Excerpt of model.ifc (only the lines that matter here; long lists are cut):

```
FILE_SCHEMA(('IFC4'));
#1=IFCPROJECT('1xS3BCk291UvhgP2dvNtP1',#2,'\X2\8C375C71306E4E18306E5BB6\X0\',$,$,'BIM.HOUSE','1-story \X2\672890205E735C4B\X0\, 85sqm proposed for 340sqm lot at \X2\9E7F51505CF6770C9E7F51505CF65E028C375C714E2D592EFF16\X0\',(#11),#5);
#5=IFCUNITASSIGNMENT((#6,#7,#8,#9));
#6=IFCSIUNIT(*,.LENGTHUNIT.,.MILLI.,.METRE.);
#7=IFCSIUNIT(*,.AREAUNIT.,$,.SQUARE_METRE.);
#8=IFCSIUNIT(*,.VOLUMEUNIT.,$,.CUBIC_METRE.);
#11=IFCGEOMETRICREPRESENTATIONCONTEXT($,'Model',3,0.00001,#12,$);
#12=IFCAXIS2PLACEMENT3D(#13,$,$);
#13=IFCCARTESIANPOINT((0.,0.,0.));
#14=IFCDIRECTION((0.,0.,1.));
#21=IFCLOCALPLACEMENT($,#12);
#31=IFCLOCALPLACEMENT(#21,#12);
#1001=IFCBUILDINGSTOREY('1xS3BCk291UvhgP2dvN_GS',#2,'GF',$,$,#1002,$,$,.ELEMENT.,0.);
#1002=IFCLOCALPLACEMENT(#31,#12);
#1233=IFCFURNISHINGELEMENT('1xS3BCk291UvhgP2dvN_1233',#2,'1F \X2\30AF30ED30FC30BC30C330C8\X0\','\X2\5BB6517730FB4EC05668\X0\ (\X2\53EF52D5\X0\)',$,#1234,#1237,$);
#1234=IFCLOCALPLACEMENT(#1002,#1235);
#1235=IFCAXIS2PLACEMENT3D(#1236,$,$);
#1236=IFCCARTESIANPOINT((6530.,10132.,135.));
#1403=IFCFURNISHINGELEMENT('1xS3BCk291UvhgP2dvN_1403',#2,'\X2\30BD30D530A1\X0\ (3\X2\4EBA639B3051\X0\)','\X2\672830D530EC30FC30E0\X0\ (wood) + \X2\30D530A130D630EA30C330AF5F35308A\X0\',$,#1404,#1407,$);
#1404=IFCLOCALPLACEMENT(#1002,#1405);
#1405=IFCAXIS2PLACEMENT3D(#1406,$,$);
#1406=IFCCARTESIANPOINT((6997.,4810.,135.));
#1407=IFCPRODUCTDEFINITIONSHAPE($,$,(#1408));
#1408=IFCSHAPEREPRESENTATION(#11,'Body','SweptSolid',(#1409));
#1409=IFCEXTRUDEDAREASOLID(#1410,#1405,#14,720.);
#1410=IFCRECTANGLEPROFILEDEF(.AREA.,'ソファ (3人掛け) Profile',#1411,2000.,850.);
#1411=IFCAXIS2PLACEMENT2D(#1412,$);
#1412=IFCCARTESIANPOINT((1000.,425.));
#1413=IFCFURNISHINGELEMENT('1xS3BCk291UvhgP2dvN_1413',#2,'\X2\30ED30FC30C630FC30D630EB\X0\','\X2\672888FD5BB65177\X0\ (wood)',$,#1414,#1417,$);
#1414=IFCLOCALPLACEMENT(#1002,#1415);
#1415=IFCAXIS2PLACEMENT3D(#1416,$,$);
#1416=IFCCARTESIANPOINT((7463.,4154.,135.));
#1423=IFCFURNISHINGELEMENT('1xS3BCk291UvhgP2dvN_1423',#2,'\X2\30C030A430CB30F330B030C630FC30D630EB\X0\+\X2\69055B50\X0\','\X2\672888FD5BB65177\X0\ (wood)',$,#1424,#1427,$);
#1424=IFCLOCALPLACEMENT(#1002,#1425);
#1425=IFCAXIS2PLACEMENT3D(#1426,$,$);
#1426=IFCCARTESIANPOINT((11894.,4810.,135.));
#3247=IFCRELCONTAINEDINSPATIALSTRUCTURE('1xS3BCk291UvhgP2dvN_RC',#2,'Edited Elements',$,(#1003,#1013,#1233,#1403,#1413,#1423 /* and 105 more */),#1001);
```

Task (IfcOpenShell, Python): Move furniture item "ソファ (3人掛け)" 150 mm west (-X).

```python
import ifcopenshell
import ifcopenshell.api.geometry
import ifcopenshell.util.placement

model = ifcopenshell.open("model.ifc")

item = model.by_guid("1xS3BCk291UvhgP2dvN_1403")
matrix = ifcopenshell.util.placement.get_local_placement(item.ObjectPlacement)
matrix[0, 3] -= 150.0
ifcopenshell.api.geometry.edit_object_placement(model, product=item, matrix=matrix, is_si=False)

print(ifcopenshell.util.placement.get_local_placement(item.ObjectPlacement).round(3) + 0.0)

model.write("model_edited.ifc")
```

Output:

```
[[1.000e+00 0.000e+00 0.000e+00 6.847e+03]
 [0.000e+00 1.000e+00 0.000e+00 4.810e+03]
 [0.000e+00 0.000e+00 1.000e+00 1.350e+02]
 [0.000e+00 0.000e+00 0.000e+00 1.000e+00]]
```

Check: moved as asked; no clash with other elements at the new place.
